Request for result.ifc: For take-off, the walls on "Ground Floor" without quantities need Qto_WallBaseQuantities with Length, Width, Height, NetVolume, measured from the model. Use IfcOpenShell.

First a look at what the model holds.

```python
import ifcopenshell
import ifcopenshell.util.element
import ifcopenshell.util.unit

model = ifcopenshell.open("result.ifc")
print(model.schema)
for unit_type in ("LENGTHUNIT", "AREAUNIT", "VOLUMEUNIT"):
    print(unit_type, ifcopenshell.util.unit.calculate_unit_scale(model, unit_type))
storey = next(s for s in model.by_type("IfcBuildingStorey") if s.Name == "Ground Floor")
walls = [e for e in ifcopenshell.util.element.get_decomposition(storey) if e.is_a("IfcWall")]
for e in sorted(walls, key=lambda e: e.id()):
    print(e.id(), e.is_a(), e.Name, list(ifcopenshell.util.element.get_psets(e, qtos_only=True)), sep=" | ")
```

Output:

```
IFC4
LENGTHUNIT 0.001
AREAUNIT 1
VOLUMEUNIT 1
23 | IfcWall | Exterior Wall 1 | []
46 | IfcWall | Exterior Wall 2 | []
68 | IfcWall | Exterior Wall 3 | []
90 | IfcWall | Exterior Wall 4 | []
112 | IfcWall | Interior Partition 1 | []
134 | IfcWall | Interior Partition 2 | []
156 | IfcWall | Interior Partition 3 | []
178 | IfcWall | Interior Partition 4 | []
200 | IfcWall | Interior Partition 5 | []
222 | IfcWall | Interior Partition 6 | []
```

```python
import ifcopenshell
import ifcopenshell.api.pset
import ifcopenshell.geom
import ifcopenshell.util.element
import ifcopenshell.util.shape
import ifcopenshell.util.unit

model = ifcopenshell.open("result.ifc")
unit_scale = ifcopenshell.util.unit.calculate_unit_scale(model)
volume_scale = ifcopenshell.util.unit.calculate_unit_scale(model, "VOLUMEUNIT")
settings = ifcopenshell.geom.settings()

storey = next(s for s in model.by_type("IfcBuildingStorey") if s.Name == "Ground Floor")
walls = [e for e in ifcopenshell.util.element.get_decomposition(storey) if e.is_a("IfcWall")]

for e in sorted(walls, key=lambda e: e.id()):
    if ifcopenshell.util.element.get_psets(e, qtos_only=True, should_inherit=False):
        continue
    # Geometry comes back in metres, in the element's own axes.
    shape = ifcopenshell.geom.create_shape(settings, e)
    values = {
        "Length": ifcopenshell.util.shape.get_x(shape.geometry) / unit_scale,
        "Width": ifcopenshell.util.shape.get_y(shape.geometry) / unit_scale,
        "Height": ifcopenshell.util.shape.get_z(shape.geometry) / unit_scale,
        "NetVolume": ifcopenshell.util.shape.get_volume(shape.geometry) / volume_scale,
    }
    qto = ifcopenshell.api.pset.add_qto(model, product=e, name="Qto_WallBaseQuantities")
    ifcopenshell.api.pset.edit_qto(model, qto=qto, properties=values)
    print(e.id(), {k: round(v, 3) for k, v in values.items()})

model.write("result_updated.ifc")
```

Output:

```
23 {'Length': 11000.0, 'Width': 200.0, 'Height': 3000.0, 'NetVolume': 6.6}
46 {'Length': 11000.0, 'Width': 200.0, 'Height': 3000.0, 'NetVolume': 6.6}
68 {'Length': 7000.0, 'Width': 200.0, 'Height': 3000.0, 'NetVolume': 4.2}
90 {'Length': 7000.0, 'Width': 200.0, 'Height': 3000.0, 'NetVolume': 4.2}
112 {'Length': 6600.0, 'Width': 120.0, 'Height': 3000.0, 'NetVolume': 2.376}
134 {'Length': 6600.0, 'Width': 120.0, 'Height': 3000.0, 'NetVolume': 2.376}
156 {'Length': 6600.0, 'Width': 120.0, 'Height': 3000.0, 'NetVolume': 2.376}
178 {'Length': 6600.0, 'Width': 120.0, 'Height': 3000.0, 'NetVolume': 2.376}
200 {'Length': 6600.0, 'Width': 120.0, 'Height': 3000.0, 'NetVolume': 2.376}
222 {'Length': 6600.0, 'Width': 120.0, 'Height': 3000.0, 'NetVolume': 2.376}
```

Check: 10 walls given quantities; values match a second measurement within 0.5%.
